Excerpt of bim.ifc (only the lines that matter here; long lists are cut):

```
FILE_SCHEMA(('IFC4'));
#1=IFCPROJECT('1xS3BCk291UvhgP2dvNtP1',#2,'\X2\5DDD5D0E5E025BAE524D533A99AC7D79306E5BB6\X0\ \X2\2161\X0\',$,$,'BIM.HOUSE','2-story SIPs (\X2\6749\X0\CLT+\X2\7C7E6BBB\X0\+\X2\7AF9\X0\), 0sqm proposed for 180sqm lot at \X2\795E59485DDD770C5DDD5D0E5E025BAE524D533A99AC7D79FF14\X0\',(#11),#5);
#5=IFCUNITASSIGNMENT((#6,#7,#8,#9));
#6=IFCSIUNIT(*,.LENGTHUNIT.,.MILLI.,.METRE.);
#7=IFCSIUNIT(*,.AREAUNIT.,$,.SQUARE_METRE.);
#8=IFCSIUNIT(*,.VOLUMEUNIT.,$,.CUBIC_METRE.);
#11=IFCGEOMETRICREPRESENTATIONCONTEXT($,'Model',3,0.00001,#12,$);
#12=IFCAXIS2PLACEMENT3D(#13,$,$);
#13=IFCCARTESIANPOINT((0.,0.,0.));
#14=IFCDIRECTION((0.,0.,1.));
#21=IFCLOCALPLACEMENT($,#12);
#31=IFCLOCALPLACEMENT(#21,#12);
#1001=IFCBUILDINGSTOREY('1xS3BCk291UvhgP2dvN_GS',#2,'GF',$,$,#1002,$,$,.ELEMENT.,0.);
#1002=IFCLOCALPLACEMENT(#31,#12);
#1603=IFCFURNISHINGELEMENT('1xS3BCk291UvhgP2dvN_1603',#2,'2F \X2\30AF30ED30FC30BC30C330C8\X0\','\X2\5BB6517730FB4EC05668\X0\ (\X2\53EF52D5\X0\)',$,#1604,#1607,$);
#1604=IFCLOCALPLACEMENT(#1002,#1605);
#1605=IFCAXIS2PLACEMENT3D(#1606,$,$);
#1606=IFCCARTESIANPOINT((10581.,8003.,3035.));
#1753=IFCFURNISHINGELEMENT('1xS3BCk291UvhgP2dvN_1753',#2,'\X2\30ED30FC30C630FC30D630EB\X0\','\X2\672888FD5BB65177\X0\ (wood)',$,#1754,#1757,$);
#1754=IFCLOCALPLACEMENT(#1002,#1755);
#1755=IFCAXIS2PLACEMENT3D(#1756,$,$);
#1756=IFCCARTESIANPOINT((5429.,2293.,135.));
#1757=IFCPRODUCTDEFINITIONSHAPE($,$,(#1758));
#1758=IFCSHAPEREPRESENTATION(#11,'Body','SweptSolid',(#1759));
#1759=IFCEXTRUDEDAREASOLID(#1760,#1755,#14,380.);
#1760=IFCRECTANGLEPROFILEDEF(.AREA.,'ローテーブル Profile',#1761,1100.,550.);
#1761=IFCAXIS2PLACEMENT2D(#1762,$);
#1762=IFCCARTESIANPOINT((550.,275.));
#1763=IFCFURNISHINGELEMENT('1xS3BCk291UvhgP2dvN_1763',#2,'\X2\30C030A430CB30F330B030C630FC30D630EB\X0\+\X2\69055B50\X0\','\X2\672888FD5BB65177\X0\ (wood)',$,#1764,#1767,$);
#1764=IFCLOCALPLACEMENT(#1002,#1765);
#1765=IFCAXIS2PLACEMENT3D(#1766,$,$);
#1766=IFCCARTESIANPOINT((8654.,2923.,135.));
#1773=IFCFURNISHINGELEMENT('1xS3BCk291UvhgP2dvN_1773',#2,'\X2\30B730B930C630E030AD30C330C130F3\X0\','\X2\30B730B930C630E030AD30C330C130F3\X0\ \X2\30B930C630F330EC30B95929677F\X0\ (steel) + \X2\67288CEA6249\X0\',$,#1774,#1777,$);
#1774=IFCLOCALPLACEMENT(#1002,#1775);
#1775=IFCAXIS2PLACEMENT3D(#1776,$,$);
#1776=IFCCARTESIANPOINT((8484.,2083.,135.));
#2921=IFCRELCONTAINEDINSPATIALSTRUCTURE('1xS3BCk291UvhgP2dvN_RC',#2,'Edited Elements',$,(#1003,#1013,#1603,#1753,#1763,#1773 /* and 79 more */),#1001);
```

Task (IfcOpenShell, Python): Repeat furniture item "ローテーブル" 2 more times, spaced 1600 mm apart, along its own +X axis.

```python
import ifcopenshell
import ifcopenshell.api.geometry
import ifcopenshell.api.root
import ifcopenshell.util.element
import ifcopenshell.util.placement
import ifcopenshell.util.unit

model = ifcopenshell.open("bim.ifc")
unit_scale = ifcopenshell.util.unit.calculate_unit_scale(model)


def reuse_history(source, copy):
    """copy_class also copies each property set's owner history, people and application; keep the originals."""
    for rel in copy.IsDefinedBy:
        if rel.is_a("IfcRelDefinesByProperties") and (history := rel.RelatingPropertyDefinition.OwnerHistory):
            rel.RelatingPropertyDefinition.OwnerHistory = source.OwnerHistory
            ifcopenshell.util.element.remove_deep2(model, history)


source = model.by_id(1753)
base = ifcopenshell.util.placement.get_local_placement(source.ObjectPlacement)
step = base[:3, 0] * 1.6 / unit_scale

for i in range(1, 3):
    copy = ifcopenshell.api.root.copy_class(model, product=source)
    copy.Representation = ifcopenshell.util.element.copy_deep(
        model, source.Representation, exclude=["IfcGeometricRepresentationContext", "IfcRepresentationMap"]
    )
    reuse_history(source, copy)
    matrix = base.copy()
    matrix[:3, 3] += i * step
    print("added at", matrix[:3, 3].round(3) + 0.0)
    ifcopenshell.api.geometry.edit_object_placement(model, product=copy, matrix=matrix, is_si=False)

model.write("bim-out.ifc")
```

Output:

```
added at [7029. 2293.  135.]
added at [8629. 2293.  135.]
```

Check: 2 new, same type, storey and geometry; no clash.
